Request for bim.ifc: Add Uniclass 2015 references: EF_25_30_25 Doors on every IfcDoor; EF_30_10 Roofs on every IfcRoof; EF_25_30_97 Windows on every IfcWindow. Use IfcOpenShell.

First a look at what the model holds.

```python
import ifcopenshell

model = ifcopenshell.open("bim.ifc")
print(model.schema)
print("classifications:", [c.Name for c in model.by_type("IfcClassification")])
for ifc_class in ("IfcDoor", "IfcRoof", "IfcStair", "IfcWall", "IfcWindow"):
    print(ifc_class, len(model.by_type(ifc_class)))
```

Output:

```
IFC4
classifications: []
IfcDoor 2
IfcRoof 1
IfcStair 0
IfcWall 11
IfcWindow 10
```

```python
import ifcopenshell
import ifcopenshell.api.classification

model = ifcopenshell.open("bim.ifc")

system = ifcopenshell.api.classification.add_classification(model, classification="Uniclass 2015")

codes = {
    "IfcDoor": ("EF_25_30_25", "Doors"),
    "IfcRoof": ("EF_30_10", "Roofs"),
    "IfcWindow": ("EF_25_30_97", "Windows"),
}
for ifc_class, (code, name) in codes.items():
    products = model.by_type(ifc_class)
    ifcopenshell.api.classification.add_reference(
        model, products=products, classification=system, identification=code, name=name
    )
    print(code, len(products))

model.write("bim_rev.ifc")
```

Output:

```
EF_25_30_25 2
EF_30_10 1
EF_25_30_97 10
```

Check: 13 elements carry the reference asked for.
